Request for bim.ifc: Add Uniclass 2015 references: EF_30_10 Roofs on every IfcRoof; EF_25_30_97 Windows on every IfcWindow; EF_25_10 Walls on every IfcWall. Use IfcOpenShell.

First a look at what the model holds.

```python
import ifcopenshell

model = ifcopenshell.open("bim.ifc")
print(model.schema)
print("classifications:", [c.Name for c in model.by_type("IfcClassification")])
for ifc_class in ("IfcDoor", "IfcRoof", "IfcStair", "IfcWall", "IfcWindow"):
    print(ifc_class, len(model.by_type(ifc_class)))
```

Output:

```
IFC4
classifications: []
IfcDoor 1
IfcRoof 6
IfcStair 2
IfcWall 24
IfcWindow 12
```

```python
import ifcopenshell
import ifcopenshell.api.classification

model = ifcopenshell.open("bim.ifc")

system = ifcopenshell.api.classification.add_classification(model, classification="Uniclass 2015")

codes = {
    "IfcRoof": ("EF_30_10", "Roofs"),
    "IfcWindow": ("EF_25_30_97", "Windows"),
    "IfcWall": ("EF_25_10", "Walls"),
}
for ifc_class, (code, name) in codes.items():
    products = model.by_type(ifc_class)
    ifcopenshell.api.classification.add_reference(
        model, products=products, classification=system, identification=code, name=name
    )
    print(code, len(products))

model.write("bim_v2.ifc")
```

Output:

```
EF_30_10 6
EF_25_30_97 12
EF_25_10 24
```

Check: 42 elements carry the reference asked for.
